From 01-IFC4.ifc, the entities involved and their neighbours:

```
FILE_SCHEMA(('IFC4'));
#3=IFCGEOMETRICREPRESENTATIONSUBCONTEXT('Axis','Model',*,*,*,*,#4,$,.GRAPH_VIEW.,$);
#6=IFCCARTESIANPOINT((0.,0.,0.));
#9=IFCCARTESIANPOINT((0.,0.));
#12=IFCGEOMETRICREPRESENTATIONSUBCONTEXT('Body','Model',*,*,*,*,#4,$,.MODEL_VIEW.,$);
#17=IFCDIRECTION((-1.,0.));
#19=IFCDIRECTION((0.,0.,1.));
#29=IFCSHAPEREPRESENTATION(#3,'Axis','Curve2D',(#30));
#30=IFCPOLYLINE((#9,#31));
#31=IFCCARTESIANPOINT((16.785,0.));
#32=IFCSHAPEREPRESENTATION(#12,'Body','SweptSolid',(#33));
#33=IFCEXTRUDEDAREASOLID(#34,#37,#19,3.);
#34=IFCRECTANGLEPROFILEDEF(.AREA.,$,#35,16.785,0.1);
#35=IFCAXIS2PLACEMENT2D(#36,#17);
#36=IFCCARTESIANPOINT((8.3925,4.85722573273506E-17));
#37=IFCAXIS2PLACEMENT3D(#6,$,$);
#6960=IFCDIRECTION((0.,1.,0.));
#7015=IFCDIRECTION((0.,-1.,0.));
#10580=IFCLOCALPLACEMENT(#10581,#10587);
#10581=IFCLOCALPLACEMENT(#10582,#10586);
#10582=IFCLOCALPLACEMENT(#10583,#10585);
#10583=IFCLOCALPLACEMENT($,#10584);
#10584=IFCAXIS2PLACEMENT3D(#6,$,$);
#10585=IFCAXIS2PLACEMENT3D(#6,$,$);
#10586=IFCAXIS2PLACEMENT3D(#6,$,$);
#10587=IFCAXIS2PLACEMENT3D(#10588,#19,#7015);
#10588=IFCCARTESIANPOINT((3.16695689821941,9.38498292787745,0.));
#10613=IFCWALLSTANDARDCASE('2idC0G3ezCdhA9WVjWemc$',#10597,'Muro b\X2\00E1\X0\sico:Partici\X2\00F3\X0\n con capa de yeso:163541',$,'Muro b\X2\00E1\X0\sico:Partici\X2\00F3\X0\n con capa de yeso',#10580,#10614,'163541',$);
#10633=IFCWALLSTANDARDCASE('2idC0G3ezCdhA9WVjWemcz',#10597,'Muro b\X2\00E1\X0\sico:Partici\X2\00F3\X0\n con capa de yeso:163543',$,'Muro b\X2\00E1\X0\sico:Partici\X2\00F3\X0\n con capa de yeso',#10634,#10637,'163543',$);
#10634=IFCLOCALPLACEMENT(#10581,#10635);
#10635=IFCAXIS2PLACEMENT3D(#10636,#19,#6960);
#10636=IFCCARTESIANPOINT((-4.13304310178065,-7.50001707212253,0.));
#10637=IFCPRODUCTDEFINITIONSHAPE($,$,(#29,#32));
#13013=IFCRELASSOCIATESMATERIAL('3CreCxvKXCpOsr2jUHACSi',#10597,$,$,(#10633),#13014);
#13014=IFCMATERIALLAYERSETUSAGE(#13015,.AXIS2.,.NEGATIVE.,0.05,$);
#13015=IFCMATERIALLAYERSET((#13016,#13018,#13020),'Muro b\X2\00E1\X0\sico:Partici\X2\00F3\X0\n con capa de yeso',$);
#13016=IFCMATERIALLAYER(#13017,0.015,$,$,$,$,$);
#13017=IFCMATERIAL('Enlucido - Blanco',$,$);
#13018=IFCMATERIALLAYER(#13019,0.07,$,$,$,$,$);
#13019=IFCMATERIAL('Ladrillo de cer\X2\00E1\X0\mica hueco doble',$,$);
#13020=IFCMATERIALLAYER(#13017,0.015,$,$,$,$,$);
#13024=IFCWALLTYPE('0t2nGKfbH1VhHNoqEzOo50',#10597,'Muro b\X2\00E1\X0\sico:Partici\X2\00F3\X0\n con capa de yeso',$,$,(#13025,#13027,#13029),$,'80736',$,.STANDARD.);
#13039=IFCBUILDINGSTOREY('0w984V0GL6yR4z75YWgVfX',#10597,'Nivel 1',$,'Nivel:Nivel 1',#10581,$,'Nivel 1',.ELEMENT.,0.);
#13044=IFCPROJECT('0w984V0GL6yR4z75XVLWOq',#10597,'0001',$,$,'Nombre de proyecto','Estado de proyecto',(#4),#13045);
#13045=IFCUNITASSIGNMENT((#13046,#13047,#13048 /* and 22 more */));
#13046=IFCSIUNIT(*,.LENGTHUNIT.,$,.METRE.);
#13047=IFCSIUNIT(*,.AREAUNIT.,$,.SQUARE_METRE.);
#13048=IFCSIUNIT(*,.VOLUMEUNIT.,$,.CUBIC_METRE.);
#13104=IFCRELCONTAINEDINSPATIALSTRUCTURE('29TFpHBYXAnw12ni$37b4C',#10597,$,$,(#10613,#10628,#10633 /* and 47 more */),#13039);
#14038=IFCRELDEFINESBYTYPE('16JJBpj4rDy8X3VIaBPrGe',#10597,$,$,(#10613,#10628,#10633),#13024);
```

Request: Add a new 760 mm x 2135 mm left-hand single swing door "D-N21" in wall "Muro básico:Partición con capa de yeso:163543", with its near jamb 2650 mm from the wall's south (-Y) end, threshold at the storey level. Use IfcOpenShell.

```python
import numpy as np
import ifcopenshell
import ifcopenshell.api.feature
import ifcopenshell.api.geometry
import ifcopenshell.api.root
import ifcopenshell.api.spatial
import ifcopenshell.geom
import ifcopenshell.util.element
import ifcopenshell.util.placement
import ifcopenshell.util.representation
import ifcopenshell.util.shape
import ifcopenshell.util.unit

model = ifcopenshell.open("01-IFC4.ifc")
unit_scale = ifcopenshell.util.unit.calculate_unit_scale(model)
settings = ifcopenshell.geom.settings()


def volume(element):
    """Net volume in cubic metres, openings subtracted."""
    shape = ifcopenshell.geom.create_shape(settings, element)
    return ifcopenshell.util.shape.get_volume(shape.geometry)


wall = model.by_guid("2idC0G3ezCdhA9WVjWemcz")
storey = ifcopenshell.util.element.get_container(wall, ifc_class="IfcBuildingStorey")
context = ifcopenshell.util.representation.get_context(model, "Model", "Body", "MODEL_VIEW")
before = volume(wall)

width, height, from_end, sill = 0.76, 2.135, 2.65, 0.0  # metres

# The wall runs along its own X axis, and the end named is its -X end.
wall_shape = ifcopenshell.geom.create_shape(settings, wall)
x, y, z = ifcopenshell.util.shape.get_vertices(wall_shape.geometry).T
start = x.min() + from_end
face, thickness = float(y.min()), float(y.max() - y.min())
wall_matrix = ifcopenshell.util.placement.get_local_placement(wall.ObjectPlacement)
level = ifcopenshell.util.placement.get_local_placement(storey.ObjectPlacement)[2, 3]


def in_wall(x, y):
    """Placement at x, y metres in the wall's axes, at sill height."""
    matrix = wall_matrix.copy()
    matrix[:, 3] = wall_matrix @ np.array([x / unit_scale, y / unit_scale, 0.0, 1.0])
    matrix[2, 3] = level + sill / unit_scale
    return matrix


# Opening: a box that overshoots both wall faces by 50 mm.
opening = ifcopenshell.api.root.create_entity(model, ifc_class="IfcOpeningElement", predefined_type="OPENING")
box = ifcopenshell.api.geometry.add_wall_representation(
    model, context=context, length=width, height=height, thickness=thickness + 0.1
)
ifcopenshell.api.geometry.assign_representation(model, product=opening, representation=box)
ifcopenshell.api.geometry.edit_object_placement(model, product=opening, matrix=in_wall(start, face - 0.05), is_si=False)
ifcopenshell.api.feature.add_feature(model, feature=opening, element=wall)

door = ifcopenshell.api.root.create_entity(model, ifc_class="IfcDoor", name="D-N21", predefined_type="DOOR")
door.OverallWidth, door.OverallHeight = width / unit_scale, height / unit_scale
door.OperationType = "SINGLE_SWING_LEFT"
body = ifcopenshell.api.geometry.add_door_representation(
    model,
    context=context,
    overall_width=door.OverallWidth,
    overall_height=door.OverallHeight,
    operation_type="SINGLE_SWING_LEFT",
    lining_properties={"LiningDepth": thickness / unit_scale, "ThresholdDepth": thickness / unit_scale},
)
ifcopenshell.api.geometry.assign_representation(model, product=door, representation=body)
ifcopenshell.api.spatial.assign_container(model, products=[door], relating_structure=storey)
ifcopenshell.api.feature.add_filling(model, opening=opening, element=door)

# The lining spans the wall, so the door starts at the wall face.
ifcopenshell.api.geometry.edit_object_placement(model, product=door, matrix=in_wall(start, face), is_si=False)

after = volume(wall)

print(f"wall volume {before:.3f} -> {after:.3f} m3")

model.write("01-IFC4_v2.ifc")
```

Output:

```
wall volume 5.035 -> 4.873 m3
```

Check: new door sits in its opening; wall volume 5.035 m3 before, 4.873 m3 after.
